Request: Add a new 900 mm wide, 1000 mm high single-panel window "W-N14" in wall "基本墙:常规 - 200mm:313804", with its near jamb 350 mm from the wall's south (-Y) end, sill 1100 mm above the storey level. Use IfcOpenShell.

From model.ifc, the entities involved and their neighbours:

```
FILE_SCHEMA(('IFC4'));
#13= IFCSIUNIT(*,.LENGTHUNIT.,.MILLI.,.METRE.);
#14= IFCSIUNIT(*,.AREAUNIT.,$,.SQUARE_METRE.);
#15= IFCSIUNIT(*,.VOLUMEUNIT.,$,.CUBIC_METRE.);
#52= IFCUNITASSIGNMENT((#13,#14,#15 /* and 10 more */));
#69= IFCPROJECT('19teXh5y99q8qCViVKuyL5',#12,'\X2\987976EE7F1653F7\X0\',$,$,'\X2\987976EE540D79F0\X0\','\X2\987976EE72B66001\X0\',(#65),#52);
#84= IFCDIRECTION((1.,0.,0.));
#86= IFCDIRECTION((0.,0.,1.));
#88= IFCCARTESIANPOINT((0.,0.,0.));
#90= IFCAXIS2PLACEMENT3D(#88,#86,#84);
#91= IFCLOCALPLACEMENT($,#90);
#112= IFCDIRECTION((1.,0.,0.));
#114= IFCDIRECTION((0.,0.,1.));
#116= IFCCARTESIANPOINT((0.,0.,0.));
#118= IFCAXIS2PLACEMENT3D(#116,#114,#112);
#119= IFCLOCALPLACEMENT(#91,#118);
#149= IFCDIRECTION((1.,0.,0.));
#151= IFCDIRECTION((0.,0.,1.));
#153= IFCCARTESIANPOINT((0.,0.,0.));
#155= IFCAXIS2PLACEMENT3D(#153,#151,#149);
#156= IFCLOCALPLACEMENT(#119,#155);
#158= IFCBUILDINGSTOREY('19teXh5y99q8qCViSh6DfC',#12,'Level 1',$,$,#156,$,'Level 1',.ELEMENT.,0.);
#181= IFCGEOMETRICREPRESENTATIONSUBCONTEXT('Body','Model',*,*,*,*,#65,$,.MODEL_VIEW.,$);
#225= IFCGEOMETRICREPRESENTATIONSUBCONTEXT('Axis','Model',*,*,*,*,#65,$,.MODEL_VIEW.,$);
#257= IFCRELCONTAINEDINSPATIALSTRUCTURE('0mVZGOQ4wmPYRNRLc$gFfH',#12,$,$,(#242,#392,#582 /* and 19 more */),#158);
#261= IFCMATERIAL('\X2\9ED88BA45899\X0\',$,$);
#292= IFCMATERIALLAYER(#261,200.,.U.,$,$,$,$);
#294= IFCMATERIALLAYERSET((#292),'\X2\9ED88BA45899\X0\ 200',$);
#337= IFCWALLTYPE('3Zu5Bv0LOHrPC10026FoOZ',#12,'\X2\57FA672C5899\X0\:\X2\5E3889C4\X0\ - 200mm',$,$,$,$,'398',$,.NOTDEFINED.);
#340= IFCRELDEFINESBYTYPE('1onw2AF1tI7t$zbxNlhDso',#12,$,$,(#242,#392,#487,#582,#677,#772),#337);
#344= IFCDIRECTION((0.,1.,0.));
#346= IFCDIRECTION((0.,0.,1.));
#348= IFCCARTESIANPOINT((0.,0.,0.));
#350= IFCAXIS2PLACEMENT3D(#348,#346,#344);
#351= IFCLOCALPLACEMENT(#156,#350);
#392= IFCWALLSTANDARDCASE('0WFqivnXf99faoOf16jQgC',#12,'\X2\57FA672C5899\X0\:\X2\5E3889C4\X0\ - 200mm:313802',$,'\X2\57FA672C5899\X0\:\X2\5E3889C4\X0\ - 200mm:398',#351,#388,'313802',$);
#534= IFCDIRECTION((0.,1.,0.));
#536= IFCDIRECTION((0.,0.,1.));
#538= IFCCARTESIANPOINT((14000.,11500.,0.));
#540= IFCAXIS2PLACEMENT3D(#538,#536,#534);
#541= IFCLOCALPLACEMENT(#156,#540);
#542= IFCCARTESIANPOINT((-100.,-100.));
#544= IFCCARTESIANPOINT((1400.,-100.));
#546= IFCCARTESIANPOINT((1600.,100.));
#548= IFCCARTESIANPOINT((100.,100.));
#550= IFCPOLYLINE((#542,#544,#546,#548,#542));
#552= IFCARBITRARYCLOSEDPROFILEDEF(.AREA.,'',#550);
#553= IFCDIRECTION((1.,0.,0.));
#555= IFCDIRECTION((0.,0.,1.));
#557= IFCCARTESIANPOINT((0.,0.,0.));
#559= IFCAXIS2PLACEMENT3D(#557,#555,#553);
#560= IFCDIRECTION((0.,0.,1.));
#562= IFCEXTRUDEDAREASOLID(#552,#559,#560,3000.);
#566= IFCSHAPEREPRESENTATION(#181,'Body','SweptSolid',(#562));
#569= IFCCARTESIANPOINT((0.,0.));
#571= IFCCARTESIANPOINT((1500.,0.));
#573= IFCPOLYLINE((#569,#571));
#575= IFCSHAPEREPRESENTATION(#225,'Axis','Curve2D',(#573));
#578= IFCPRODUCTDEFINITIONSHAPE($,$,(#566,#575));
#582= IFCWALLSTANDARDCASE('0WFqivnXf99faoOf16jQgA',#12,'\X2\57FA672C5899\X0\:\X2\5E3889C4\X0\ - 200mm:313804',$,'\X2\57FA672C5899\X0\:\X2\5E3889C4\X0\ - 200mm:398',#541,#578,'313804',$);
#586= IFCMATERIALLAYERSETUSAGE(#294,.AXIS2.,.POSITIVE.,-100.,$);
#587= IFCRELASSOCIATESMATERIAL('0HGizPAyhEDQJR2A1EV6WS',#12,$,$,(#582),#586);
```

```python
import numpy as np
import ifcopenshell
import ifcopenshell.api.feature
import ifcopenshell.api.geometry
import ifcopenshell.api.root
import ifcopenshell.api.spatial
import ifcopenshell.geom
import ifcopenshell.util.element
import ifcopenshell.util.placement
import ifcopenshell.util.representation
import ifcopenshell.util.shape
import ifcopenshell.util.unit

model = ifcopenshell.open("model.ifc")
unit_scale = ifcopenshell.util.unit.calculate_unit_scale(model)
settings = ifcopenshell.geom.settings()


def volume(element):
    """Net volume in cubic metres, openings subtracted."""
    shape = ifcopenshell.geom.create_shape(settings, element)
    return ifcopenshell.util.shape.get_volume(shape.geometry)


wall = model.by_guid("0WFqivnXf99faoOf16jQgA")
storey = ifcopenshell.util.element.get_container(wall, ifc_class="IfcBuildingStorey")
context = ifcopenshell.util.representation.get_context(model, "Model", "Body", "MODEL_VIEW")
before = volume(wall)

width, height, from_end, sill = 0.9, 1, 0.35, 1.1  # metres

# The wall runs along its own X axis, and the end named is its -X end.
wall_shape = ifcopenshell.geom.create_shape(settings, wall)
x, y, z = ifcopenshell.util.shape.get_vertices(wall_shape.geometry).T
start = x.min() + from_end
face, thickness = float(y.min()), float(y.max() - y.min())
wall_matrix = ifcopenshell.util.placement.get_local_placement(wall.ObjectPlacement)
level = ifcopenshell.util.placement.get_local_placement(storey.ObjectPlacement)[2, 3]


def in_wall(x, y):
    """Placement at x, y metres in the wall's axes, at sill height."""
    matrix = wall_matrix.copy()
    matrix[:, 3] = wall_matrix @ np.array([x / unit_scale, y / unit_scale, 0.0, 1.0])
    matrix[2, 3] = level + sill / unit_scale
    return matrix


# Opening: a box that overshoots both wall faces by 50 mm.
opening = ifcopenshell.api.root.create_entity(model, ifc_class="IfcOpeningElement", predefined_type="OPENING")
box = ifcopenshell.api.geometry.add_wall_representation(
    model, context=context, length=width, height=height, thickness=thickness + 0.1
)
ifcopenshell.api.geometry.assign_representation(model, product=opening, representation=box)
ifcopenshell.api.geometry.edit_object_placement(model, product=opening, matrix=in_wall(start, face - 0.05), is_si=False)
ifcopenshell.api.feature.add_feature(model, feature=opening, element=wall)

window = ifcopenshell.api.root.create_entity(model, ifc_class="IfcWindow", name="W-N14", predefined_type="WINDOW")
window.OverallWidth, window.OverallHeight = width / unit_scale, height / unit_scale
window.PartitioningType = "SINGLE_PANEL"
body = ifcopenshell.api.geometry.add_window_representation(
    model,
    context=context,
    overall_width=window.OverallWidth,
    overall_height=window.OverallHeight,
    partition_type="SINGLE_PANEL",
)
ifcopenshell.api.geometry.assign_representation(model, product=window, representation=body)
ifcopenshell.api.spatial.assign_container(model, products=[window], relating_structure=storey)
ifcopenshell.api.feature.add_filling(model, opening=opening, element=window)

# Centre the window in the wall's thickness.
ifcopenshell.api.geometry.edit_object_placement(model, product=window, matrix=in_wall(start, face), is_si=False)
window_shape = ifcopenshell.geom.create_shape(settings, window)
depth = ifcopenshell.util.shape.get_vertices(window_shape.geometry)[:, 1]
offset = face + thickness / 2 - (depth.min() + depth.max()) / 2
ifcopenshell.api.geometry.edit_object_placement(model, product=window, matrix=in_wall(start, offset), is_si=False)

after = volume(wall)

print(f"wall volume {before:.3f} -> {after:.3f} m3")

model.write("model_rev.ifc")
```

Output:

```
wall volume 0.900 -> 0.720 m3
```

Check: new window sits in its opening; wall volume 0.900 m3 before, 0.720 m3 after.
